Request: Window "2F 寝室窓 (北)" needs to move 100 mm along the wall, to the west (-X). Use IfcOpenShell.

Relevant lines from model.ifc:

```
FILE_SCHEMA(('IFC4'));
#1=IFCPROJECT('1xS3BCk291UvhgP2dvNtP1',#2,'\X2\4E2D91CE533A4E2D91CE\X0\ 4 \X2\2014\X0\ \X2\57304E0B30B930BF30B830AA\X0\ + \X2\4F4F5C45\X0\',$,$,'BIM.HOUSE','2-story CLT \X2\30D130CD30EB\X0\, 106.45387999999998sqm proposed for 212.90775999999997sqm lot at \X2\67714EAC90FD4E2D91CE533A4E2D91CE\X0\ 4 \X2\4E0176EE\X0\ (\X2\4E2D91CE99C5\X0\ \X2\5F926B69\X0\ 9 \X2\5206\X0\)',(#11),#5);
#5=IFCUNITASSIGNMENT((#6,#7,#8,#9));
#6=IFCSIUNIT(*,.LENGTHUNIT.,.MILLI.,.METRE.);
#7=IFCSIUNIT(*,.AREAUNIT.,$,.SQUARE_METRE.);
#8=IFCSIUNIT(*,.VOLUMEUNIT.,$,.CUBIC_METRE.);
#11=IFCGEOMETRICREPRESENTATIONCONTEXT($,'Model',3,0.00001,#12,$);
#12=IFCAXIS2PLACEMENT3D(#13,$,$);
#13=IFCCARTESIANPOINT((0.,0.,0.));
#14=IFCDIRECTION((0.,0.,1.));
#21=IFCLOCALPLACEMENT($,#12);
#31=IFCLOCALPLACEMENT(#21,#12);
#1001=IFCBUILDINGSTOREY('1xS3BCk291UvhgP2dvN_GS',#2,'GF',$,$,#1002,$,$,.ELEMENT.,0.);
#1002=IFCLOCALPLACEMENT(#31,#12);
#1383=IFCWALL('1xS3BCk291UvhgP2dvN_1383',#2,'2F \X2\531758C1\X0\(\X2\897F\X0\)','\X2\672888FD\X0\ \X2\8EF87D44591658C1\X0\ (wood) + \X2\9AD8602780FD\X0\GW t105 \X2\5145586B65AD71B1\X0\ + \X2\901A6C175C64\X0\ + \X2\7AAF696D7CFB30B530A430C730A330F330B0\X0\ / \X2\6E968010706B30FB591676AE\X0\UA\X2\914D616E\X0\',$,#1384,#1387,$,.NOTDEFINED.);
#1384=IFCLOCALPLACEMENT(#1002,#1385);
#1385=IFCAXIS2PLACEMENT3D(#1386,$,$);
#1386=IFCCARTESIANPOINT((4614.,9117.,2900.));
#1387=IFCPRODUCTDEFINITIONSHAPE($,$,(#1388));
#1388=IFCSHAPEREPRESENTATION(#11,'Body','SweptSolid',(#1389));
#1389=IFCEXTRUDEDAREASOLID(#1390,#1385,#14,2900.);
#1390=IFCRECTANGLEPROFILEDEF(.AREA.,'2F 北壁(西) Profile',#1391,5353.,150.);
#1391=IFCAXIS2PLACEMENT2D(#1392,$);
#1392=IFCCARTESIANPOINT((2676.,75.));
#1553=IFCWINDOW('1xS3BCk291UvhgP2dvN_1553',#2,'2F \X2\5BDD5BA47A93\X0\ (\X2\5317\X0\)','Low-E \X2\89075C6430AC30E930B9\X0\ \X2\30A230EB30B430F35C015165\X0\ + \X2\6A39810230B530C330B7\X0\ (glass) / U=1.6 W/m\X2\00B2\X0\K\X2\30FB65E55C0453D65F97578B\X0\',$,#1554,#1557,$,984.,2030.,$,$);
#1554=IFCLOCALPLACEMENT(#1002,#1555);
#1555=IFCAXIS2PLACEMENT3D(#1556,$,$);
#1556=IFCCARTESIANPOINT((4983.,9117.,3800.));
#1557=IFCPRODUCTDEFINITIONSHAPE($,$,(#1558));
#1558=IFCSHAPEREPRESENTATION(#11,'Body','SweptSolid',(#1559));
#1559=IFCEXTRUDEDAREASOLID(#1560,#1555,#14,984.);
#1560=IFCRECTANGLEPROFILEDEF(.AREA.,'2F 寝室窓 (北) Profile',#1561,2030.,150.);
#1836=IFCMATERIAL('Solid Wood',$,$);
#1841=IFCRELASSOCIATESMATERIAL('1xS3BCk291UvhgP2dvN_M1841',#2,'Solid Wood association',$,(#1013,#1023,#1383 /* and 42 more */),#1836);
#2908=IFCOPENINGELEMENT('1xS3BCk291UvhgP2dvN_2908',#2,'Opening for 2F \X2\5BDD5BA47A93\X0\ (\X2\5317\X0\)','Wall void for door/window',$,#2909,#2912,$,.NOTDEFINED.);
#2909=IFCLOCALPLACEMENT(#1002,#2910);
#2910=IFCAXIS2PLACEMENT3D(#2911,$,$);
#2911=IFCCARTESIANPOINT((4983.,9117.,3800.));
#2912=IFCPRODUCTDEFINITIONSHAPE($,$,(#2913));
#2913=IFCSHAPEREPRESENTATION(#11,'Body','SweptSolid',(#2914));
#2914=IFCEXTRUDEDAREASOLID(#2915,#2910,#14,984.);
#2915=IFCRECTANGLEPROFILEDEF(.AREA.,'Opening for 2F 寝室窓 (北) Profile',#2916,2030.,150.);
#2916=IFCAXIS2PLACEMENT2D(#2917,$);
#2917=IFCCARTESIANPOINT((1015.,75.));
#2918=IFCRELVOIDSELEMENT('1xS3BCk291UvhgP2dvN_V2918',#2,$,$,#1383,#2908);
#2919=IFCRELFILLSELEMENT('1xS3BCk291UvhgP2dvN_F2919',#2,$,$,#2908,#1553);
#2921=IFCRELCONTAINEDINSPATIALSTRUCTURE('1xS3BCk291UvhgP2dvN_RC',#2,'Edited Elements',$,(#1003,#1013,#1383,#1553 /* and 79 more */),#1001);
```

```python
import ifcopenshell
import ifcopenshell.api.geometry
import ifcopenshell.util.placement

model = ifcopenshell.open("model.ifc")

window = model.by_id(1553)
opening = window.FillsVoids[0].RelatingOpeningElement
wall = opening.VoidsElements[0].RelatingBuildingElement

wall_matrix = ifcopenshell.util.placement.get_local_placement(wall.ObjectPlacement)
shift = wall_matrix[:3, 0] * -100.0
before = ifcopenshell.util.placement.get_local_placement(window.ObjectPlacement)[:3, 3].copy()

# The window is not placed relative to its opening, so move both.
for product in (opening, window):
    matrix = ifcopenshell.util.placement.get_local_placement(product.ObjectPlacement)
    matrix[:3, 3] += shift
    ifcopenshell.api.geometry.edit_object_placement(model, product=product, matrix=matrix, is_si=False)

after = ifcopenshell.util.placement.get_local_placement(window.ObjectPlacement)[:3, 3]
print("window moved by", (after - before).round(3) + 0.0)

model.write("model_v2.ifc")
```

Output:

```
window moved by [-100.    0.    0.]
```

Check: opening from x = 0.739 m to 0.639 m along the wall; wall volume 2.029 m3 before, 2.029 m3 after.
